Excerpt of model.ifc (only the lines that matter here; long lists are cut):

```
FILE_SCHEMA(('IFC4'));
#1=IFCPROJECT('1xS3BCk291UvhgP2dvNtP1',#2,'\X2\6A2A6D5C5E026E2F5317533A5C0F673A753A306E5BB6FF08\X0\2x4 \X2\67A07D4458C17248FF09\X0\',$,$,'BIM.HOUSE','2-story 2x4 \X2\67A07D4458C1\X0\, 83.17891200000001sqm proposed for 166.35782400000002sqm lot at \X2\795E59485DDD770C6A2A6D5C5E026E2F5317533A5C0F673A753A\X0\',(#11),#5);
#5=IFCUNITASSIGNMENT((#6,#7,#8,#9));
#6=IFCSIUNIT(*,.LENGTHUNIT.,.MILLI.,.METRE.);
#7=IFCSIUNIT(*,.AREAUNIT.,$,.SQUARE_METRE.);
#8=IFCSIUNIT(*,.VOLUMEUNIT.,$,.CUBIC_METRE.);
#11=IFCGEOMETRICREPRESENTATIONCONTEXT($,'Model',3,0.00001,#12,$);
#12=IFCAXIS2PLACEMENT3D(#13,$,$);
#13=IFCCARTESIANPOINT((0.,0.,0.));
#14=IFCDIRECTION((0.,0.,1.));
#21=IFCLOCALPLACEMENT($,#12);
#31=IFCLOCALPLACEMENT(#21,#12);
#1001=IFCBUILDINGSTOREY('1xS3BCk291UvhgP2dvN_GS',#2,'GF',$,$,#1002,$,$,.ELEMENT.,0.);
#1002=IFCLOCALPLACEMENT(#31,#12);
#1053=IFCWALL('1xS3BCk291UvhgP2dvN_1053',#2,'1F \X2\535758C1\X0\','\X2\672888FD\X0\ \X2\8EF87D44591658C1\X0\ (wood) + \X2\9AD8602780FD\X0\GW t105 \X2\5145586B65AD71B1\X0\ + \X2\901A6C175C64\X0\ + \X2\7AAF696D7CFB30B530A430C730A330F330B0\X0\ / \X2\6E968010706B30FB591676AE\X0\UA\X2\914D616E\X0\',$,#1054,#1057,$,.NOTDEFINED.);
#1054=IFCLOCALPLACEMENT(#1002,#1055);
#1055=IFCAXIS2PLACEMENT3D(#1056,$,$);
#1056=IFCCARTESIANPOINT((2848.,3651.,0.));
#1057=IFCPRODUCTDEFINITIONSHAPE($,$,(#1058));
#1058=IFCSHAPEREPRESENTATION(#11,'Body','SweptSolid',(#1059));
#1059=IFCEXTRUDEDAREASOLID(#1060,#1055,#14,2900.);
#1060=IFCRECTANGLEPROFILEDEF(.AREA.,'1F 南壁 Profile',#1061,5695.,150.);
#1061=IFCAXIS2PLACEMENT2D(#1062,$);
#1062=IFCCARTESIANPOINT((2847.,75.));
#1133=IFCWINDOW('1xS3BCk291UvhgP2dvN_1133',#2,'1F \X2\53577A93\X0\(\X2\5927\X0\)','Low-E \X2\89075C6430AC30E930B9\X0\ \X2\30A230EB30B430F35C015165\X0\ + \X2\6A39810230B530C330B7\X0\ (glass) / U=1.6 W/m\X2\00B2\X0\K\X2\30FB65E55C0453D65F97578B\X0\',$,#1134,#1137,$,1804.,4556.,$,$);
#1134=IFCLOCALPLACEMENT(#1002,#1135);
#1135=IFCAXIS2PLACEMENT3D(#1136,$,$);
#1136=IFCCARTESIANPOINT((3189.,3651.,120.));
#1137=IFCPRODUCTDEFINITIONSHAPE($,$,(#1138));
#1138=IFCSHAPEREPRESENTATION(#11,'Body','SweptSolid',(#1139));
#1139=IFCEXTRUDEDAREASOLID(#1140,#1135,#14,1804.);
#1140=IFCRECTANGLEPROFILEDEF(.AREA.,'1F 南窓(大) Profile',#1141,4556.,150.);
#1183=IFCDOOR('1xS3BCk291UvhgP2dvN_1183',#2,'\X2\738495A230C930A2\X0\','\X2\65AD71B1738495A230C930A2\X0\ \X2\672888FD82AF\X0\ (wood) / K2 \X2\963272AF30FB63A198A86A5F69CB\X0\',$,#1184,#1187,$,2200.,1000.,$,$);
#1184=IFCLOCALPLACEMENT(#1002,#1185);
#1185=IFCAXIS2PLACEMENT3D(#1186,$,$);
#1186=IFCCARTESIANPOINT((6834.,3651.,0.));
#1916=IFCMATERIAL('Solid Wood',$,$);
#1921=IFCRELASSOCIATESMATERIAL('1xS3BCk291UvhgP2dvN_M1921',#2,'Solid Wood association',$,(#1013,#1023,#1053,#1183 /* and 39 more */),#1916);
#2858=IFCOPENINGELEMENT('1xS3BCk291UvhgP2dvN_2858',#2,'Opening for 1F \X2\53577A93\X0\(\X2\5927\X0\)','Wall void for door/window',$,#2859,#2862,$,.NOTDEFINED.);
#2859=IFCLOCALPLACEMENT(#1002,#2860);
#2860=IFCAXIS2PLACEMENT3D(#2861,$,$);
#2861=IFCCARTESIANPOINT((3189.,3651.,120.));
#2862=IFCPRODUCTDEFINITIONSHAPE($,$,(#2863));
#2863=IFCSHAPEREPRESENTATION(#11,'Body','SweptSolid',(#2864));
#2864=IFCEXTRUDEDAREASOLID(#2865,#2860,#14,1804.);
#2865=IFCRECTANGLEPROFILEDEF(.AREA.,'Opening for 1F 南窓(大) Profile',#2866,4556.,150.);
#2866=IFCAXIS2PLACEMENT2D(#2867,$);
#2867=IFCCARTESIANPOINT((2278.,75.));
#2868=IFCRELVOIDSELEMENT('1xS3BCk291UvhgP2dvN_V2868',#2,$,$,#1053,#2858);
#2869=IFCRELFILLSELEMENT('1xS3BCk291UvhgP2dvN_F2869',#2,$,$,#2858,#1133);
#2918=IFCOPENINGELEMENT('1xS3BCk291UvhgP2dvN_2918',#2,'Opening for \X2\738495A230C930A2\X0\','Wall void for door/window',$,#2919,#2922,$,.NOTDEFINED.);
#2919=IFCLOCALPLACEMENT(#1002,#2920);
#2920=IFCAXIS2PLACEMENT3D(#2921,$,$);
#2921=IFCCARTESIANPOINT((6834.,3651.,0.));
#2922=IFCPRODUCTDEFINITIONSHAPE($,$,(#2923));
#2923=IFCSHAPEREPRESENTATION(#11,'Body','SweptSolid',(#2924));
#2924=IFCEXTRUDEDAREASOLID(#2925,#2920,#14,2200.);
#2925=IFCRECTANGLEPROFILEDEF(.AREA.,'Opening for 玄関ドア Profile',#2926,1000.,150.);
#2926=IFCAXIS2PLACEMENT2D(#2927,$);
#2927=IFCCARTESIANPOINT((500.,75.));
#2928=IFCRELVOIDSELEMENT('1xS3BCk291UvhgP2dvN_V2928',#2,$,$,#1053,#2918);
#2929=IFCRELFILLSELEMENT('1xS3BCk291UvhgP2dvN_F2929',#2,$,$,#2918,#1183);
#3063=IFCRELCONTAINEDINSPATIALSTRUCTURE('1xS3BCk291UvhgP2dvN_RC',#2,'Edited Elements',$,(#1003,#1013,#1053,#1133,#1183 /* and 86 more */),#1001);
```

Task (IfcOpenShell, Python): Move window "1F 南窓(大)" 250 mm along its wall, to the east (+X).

```python
import ifcopenshell
import ifcopenshell.api.geometry
import ifcopenshell.util.placement
import ifcopenshell.util.unit

model = ifcopenshell.open("model.ifc")
unit_scale = ifcopenshell.util.unit.calculate_unit_scale(model)

window = model.by_id(1133)
opening = window.FillsVoids[0].RelatingOpeningElement
wall = opening.VoidsElements[0].RelatingBuildingElement

wall_matrix = ifcopenshell.util.placement.get_local_placement(wall.ObjectPlacement)
shift = wall_matrix[:3, 0] * 0.25 / unit_scale
before = ifcopenshell.util.placement.get_local_placement(window.ObjectPlacement)[:3, 3].copy()

# The window is not placed relative to its opening, so move both.
for product in (opening, window):
    matrix = ifcopenshell.util.placement.get_local_placement(product.ObjectPlacement)
    matrix[:3, 3] += shift
    ifcopenshell.api.geometry.edit_object_placement(model, product=product, matrix=matrix, is_si=False)

after = ifcopenshell.util.placement.get_local_placement(window.ObjectPlacement)[:3, 3]
print("window moved by", (after - before).round(3) + 0.0)

model.write("model_edited.ifc")
```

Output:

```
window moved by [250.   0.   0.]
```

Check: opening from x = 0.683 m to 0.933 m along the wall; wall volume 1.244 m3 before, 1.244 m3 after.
